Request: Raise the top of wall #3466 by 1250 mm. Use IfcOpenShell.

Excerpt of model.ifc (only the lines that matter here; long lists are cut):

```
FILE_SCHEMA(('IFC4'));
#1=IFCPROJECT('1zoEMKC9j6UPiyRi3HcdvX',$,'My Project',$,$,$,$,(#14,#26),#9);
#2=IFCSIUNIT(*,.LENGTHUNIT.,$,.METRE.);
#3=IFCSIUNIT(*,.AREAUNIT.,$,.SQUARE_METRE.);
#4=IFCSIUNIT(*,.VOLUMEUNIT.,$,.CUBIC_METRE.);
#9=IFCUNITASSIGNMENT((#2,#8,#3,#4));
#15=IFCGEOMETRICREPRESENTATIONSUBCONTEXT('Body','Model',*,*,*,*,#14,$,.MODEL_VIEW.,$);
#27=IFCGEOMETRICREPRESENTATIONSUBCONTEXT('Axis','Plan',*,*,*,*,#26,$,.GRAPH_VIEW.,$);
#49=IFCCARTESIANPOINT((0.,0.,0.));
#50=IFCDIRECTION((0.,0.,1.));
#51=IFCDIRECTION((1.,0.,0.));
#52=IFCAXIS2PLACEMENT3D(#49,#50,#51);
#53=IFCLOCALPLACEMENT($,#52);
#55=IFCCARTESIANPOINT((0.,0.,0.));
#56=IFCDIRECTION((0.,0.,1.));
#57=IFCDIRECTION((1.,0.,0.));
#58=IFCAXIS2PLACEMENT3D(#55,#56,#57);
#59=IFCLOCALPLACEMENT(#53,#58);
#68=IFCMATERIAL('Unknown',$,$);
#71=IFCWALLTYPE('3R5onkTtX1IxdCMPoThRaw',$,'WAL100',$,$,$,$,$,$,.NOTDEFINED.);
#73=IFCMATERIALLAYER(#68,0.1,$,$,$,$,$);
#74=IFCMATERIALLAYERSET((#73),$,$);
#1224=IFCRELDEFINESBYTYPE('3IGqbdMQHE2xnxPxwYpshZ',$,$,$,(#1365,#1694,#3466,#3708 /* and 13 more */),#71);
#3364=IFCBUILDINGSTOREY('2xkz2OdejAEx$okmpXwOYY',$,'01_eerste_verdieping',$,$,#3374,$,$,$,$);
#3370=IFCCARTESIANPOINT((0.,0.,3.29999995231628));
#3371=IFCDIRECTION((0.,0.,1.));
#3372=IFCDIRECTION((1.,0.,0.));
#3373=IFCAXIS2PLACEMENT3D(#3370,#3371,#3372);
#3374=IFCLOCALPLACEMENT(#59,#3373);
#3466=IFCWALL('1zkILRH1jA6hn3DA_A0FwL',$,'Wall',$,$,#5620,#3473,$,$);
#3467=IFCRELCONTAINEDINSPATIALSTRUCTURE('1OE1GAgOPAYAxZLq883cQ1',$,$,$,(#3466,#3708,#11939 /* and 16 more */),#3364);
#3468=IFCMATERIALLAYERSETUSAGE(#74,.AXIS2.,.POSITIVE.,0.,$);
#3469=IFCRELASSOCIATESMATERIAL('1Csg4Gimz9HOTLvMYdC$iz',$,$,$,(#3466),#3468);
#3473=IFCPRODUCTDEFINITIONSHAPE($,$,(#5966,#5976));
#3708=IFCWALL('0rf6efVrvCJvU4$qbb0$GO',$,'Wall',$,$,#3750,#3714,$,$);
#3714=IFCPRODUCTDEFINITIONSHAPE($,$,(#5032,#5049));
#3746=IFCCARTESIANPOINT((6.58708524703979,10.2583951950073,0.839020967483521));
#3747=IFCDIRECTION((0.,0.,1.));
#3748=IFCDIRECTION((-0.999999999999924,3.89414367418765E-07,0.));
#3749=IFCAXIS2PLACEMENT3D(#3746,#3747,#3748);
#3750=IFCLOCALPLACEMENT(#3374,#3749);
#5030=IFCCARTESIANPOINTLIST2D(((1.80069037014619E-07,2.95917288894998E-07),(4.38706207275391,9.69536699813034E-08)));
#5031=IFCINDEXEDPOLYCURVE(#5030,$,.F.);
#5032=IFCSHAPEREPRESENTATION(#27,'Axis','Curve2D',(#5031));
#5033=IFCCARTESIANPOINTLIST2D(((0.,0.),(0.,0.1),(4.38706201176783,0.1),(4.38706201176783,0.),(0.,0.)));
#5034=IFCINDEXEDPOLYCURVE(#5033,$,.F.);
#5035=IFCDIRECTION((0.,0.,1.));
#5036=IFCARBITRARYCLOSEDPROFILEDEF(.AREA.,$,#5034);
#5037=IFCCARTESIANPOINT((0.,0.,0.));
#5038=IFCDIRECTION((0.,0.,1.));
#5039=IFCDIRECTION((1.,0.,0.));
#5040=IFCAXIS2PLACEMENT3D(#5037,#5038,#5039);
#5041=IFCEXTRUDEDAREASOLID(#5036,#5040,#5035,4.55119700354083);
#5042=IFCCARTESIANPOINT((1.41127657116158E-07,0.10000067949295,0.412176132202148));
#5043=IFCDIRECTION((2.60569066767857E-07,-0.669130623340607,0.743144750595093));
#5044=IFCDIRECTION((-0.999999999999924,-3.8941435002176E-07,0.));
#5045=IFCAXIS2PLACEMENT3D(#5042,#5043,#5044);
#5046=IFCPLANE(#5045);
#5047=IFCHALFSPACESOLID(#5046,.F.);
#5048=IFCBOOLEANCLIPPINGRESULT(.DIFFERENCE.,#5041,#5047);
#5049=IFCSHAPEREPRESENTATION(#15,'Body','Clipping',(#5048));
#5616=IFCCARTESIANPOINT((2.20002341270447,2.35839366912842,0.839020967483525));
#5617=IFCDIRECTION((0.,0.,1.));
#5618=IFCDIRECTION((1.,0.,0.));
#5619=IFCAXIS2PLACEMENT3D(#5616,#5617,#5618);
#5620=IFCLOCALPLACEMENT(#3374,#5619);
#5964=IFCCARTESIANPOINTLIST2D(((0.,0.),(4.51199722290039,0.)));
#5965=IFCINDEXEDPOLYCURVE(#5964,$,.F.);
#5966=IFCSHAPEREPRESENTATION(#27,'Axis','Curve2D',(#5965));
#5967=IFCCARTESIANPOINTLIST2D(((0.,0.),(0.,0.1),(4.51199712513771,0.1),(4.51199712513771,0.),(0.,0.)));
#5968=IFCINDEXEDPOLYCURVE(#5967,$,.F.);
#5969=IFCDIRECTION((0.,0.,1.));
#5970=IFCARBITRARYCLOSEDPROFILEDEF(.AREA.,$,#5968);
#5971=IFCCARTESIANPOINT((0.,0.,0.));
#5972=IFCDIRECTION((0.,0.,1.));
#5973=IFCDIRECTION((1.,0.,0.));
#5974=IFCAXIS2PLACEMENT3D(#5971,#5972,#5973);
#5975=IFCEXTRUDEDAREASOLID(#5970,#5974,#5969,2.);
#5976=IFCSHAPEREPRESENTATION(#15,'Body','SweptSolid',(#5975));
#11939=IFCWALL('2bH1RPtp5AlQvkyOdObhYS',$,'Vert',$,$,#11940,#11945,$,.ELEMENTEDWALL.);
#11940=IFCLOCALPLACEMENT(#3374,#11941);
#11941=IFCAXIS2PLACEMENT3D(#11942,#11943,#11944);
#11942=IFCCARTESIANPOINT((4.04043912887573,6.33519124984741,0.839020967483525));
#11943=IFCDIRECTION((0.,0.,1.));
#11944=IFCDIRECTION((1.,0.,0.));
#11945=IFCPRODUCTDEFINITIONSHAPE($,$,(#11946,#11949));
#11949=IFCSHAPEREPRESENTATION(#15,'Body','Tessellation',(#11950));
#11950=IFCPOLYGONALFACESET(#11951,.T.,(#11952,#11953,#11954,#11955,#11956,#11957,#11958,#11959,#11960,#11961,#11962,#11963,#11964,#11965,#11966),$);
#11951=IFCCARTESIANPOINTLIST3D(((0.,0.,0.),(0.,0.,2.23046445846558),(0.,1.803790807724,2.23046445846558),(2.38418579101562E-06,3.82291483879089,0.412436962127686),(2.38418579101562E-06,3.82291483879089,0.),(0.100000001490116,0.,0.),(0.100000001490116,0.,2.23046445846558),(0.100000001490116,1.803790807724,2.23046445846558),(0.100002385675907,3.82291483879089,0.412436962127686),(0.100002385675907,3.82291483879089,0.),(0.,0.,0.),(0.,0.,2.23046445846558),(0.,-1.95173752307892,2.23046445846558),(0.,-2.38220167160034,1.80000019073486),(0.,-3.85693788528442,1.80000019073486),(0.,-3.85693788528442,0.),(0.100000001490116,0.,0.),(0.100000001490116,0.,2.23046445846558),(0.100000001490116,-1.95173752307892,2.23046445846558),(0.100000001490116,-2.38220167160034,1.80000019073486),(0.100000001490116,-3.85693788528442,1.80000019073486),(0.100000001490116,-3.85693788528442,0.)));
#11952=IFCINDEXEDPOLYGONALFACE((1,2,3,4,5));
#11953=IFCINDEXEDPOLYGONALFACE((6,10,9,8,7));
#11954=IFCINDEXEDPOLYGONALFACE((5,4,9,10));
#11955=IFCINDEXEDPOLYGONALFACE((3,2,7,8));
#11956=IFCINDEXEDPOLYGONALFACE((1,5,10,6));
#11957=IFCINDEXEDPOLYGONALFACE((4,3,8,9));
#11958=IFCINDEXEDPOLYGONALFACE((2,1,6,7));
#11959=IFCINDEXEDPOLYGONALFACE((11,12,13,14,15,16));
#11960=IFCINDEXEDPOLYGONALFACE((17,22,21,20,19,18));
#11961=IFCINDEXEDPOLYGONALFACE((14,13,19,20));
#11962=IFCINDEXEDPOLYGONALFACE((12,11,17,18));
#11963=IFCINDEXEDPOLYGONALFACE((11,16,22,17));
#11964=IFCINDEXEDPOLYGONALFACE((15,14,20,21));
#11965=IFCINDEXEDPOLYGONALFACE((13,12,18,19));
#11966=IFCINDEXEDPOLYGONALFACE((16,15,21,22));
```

```python
import ifcopenshell
import ifcopenshell.geom
import ifcopenshell.util.representation
import ifcopenshell.util.shape
import ifcopenshell.util.unit

model = ifcopenshell.open("model.ifc")
unit_scale = ifcopenshell.util.unit.calculate_unit_scale(model)
settings = ifcopenshell.geom.settings()


def volume(element):
    """Net volume in cubic metres, openings subtracted."""
    shape = ifcopenshell.geom.create_shape(settings, element)
    return ifcopenshell.util.shape.get_volume(shape.geometry)


wall = model.by_id(3466)
before = volume(wall)

body = ifcopenshell.util.representation.get_representation(wall, "Model", "Body")
solid = body.Items[0]
old_height = solid.Depth
solid.Depth += 1.25 / unit_scale
after = volume(wall)

print(f"height {old_height:g} -> {solid.Depth:g}, volume {before:.3f} -> {after:.3f} m3")

model.write("model_updated.ifc")
```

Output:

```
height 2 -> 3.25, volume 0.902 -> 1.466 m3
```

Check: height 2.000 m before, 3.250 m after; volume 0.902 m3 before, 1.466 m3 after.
